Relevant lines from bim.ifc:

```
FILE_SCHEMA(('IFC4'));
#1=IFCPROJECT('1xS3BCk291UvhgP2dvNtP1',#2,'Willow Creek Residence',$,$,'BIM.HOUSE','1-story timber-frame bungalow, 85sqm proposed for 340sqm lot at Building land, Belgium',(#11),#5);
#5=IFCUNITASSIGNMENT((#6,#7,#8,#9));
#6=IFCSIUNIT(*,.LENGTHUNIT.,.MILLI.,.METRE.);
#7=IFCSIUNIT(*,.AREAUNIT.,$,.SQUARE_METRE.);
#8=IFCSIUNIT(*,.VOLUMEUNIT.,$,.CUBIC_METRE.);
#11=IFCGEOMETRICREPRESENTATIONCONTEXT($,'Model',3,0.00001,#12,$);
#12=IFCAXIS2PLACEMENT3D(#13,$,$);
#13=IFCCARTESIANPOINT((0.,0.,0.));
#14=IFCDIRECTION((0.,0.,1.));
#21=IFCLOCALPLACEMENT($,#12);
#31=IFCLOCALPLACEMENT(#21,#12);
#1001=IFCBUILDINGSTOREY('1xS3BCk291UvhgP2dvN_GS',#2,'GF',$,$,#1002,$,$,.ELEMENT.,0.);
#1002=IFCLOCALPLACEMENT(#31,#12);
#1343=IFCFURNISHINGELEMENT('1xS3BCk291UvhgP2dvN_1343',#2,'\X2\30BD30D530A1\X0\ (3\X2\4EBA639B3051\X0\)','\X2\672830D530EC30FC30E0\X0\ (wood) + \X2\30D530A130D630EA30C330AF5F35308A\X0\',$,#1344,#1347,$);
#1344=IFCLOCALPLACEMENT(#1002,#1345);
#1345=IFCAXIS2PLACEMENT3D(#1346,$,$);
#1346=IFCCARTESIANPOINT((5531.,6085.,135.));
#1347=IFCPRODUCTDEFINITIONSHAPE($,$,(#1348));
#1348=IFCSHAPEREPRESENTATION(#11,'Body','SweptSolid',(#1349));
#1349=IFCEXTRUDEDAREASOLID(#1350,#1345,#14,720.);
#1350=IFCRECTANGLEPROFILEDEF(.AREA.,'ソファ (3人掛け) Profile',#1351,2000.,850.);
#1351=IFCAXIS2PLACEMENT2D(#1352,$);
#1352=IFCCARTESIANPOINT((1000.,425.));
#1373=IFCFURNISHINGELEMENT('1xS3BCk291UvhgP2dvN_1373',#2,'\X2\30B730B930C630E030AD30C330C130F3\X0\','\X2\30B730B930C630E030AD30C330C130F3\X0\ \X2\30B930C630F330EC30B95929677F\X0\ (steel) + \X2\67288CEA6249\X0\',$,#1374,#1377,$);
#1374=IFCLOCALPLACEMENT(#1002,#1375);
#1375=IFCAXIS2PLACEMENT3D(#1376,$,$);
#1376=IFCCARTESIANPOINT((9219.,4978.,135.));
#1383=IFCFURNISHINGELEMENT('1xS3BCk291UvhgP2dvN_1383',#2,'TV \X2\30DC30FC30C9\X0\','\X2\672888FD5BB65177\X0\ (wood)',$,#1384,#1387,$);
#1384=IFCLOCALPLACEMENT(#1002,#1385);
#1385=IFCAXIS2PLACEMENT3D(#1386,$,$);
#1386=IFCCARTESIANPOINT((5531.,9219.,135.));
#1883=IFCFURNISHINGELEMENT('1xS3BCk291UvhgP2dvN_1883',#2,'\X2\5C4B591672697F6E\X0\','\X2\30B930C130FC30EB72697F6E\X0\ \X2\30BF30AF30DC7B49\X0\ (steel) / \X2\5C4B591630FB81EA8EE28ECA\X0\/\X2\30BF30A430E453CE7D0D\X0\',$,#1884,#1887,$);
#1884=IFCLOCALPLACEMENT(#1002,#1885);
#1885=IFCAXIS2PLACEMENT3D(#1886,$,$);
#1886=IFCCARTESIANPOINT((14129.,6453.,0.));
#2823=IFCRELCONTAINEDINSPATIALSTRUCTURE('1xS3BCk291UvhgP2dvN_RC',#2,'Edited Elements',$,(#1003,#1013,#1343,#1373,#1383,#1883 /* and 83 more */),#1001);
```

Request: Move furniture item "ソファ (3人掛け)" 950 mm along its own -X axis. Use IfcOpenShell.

```python
import ifcopenshell
import ifcopenshell.api.geometry
import ifcopenshell.util.placement

model = ifcopenshell.open("bim.ifc")

item = model.by_id(1343)
matrix = ifcopenshell.util.placement.get_local_placement(item.ObjectPlacement)
matrix[:3, 3] -= matrix[:3, 0] * 950.0
ifcopenshell.api.geometry.edit_object_placement(model, product=item, matrix=matrix, is_si=False)

print(ifcopenshell.util.placement.get_local_placement(item.ObjectPlacement).round(3) + 0.0)

model.write("bim-out.ifc")
```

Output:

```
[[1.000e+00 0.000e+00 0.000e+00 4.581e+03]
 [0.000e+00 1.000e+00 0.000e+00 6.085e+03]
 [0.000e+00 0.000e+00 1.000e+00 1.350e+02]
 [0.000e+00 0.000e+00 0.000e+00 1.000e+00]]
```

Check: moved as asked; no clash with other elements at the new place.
